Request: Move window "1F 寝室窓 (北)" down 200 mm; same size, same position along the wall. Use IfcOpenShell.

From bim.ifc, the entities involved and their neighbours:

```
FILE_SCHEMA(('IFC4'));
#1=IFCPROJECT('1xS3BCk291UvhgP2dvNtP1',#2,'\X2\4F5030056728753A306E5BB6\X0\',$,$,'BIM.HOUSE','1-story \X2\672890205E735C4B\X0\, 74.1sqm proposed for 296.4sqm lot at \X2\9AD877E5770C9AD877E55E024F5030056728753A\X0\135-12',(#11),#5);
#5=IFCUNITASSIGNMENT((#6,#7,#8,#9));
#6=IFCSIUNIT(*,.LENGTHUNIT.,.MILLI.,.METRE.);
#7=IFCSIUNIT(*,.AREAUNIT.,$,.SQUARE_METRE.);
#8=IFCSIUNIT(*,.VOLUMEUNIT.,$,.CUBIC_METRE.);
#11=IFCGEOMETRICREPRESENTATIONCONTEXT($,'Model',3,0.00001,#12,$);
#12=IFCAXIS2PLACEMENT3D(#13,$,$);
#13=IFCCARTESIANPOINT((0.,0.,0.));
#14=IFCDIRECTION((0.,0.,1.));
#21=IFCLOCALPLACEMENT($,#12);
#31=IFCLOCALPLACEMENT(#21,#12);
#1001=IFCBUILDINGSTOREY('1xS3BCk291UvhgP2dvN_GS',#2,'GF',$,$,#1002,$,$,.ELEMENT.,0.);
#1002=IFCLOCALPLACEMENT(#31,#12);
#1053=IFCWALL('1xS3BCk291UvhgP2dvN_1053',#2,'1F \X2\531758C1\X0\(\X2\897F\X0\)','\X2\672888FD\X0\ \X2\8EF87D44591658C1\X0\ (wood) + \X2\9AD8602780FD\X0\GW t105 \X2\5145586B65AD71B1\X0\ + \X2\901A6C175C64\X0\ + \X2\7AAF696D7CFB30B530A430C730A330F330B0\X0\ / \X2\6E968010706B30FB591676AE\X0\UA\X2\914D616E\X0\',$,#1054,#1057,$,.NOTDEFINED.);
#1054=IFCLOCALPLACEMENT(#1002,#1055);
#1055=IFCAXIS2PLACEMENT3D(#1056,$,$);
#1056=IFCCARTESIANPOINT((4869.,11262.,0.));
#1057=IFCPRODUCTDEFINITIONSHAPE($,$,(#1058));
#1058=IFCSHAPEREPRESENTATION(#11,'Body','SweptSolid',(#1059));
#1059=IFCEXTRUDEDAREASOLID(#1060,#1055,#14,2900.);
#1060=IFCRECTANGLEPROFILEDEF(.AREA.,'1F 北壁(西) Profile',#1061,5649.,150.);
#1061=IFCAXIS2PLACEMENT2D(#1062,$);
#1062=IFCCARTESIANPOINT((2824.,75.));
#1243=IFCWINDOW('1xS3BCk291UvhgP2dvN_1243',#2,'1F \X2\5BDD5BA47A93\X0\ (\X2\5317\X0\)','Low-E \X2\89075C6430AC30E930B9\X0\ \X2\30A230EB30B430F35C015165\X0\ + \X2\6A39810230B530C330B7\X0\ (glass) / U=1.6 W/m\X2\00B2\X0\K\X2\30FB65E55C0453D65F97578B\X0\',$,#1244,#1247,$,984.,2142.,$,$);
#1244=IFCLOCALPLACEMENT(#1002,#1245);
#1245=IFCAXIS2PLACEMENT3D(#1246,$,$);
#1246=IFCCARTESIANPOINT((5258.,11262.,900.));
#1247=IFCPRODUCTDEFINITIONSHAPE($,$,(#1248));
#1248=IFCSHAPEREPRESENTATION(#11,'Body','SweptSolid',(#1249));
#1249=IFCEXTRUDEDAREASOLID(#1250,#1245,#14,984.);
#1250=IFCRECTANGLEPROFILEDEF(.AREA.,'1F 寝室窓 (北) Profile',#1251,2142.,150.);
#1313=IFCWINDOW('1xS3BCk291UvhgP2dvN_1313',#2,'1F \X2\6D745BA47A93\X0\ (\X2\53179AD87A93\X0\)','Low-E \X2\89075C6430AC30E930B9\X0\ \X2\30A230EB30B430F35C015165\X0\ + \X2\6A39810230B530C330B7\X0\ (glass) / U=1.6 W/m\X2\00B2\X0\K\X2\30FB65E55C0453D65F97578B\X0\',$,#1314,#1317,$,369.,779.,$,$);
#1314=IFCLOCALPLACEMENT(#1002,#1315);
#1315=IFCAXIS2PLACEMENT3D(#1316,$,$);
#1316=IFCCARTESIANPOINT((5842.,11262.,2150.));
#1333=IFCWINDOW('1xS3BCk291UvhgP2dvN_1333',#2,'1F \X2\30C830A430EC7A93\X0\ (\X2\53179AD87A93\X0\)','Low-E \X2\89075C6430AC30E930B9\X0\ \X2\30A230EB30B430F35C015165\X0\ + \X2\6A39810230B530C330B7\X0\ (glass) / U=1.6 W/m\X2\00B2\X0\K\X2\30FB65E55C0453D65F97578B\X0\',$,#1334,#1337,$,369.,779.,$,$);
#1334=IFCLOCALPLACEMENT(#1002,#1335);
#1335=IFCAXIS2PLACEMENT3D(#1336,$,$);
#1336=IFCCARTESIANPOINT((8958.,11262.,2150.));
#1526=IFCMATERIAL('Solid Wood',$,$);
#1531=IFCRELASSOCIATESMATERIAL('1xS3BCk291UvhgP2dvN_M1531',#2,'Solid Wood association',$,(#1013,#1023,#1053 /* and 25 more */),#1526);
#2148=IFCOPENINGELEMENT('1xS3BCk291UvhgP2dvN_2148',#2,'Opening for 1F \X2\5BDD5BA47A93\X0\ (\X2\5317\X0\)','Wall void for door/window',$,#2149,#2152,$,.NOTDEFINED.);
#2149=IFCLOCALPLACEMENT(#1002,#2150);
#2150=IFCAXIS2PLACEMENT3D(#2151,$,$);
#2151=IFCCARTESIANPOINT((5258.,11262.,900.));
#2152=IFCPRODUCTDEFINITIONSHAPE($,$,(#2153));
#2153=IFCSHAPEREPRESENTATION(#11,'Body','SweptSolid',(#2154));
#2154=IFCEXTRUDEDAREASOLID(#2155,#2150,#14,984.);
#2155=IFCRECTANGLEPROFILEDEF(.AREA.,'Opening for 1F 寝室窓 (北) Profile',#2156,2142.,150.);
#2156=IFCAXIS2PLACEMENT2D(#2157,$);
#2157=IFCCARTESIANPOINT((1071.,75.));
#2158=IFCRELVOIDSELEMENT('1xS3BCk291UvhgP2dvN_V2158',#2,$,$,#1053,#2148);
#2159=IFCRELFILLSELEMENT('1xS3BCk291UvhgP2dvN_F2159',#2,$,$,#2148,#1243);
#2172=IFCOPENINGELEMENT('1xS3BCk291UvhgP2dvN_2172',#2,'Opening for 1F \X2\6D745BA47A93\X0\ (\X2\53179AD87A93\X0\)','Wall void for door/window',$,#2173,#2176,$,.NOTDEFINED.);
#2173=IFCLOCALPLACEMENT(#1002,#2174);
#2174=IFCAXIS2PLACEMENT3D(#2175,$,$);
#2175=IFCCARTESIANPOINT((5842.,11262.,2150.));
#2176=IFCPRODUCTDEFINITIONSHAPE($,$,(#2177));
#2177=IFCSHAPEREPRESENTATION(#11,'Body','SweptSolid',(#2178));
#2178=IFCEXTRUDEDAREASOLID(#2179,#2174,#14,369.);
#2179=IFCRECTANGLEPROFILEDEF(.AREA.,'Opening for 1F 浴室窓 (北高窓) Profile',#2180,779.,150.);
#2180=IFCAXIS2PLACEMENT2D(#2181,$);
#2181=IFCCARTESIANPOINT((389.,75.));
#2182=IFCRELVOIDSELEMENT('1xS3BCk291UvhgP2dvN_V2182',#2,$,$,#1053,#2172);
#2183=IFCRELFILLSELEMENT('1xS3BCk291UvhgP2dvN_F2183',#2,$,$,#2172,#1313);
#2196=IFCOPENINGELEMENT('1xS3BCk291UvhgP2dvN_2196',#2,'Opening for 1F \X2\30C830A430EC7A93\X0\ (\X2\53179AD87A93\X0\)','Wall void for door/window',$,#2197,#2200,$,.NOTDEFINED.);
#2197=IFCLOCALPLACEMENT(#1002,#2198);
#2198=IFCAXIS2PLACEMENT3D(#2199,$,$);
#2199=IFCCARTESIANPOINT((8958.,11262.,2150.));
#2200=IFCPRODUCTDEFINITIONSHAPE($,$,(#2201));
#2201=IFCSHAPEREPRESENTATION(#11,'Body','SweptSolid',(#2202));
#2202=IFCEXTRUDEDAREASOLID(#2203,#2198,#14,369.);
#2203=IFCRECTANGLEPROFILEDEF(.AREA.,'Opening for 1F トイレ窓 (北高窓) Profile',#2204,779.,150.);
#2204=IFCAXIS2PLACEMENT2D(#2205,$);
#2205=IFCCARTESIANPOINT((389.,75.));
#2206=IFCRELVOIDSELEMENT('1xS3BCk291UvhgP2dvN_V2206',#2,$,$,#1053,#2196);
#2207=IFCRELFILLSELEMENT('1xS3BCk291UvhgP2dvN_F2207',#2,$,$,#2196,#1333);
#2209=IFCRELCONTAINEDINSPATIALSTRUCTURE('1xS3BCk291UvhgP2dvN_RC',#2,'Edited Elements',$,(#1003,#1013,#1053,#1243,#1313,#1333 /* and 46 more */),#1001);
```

```python
import numpy as np
import ifcopenshell
import ifcopenshell.api.geometry
import ifcopenshell.util.placement
import ifcopenshell.util.unit

model = ifcopenshell.open("bim.ifc")
unit_scale = ifcopenshell.util.unit.calculate_unit_scale(model)

window = model.by_id(1243)
opening = window.FillsVoids[0].RelatingOpeningElement
dz = -200.0

shift = np.array([0.0, 0.0, dz])
# The window is not placed relative to its opening, so move both.
for product in (opening, window):
    matrix = ifcopenshell.util.placement.get_local_placement(product.ObjectPlacement)
    matrix[:3, 3] += shift
    ifcopenshell.api.geometry.edit_object_placement(model, product=product, matrix=matrix, is_si=False)

print(f"moved by {dz * unit_scale:+.3f} m")

model.write("bim_rev.ifc")
```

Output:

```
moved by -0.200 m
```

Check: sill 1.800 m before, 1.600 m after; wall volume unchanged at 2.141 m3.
